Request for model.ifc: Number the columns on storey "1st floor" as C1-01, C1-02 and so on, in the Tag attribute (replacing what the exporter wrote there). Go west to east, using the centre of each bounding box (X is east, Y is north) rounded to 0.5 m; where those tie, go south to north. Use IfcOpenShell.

First a look at what the model holds.

```python
import ifcopenshell
import ifcopenshell.util.element
import ifcopenshell.util.placement

model = ifcopenshell.open("model.ifc")
print(model.schema)
storey = next(s for s in model.by_type("IfcBuildingStorey") if s.Name == "1st floor")
columns = [e for e in ifcopenshell.util.element.get_decomposition(storey) if e.is_a("IfcColumn")]
for e in sorted(columns, key=lambda e: e.id()):
    origin = ifcopenshell.util.placement.get_local_placement(e.ObjectPlacement)[:3, 3]
    print(e.id(), e.Tag, e.Name, origin.round(2) + 0.0, sep=" | ")
```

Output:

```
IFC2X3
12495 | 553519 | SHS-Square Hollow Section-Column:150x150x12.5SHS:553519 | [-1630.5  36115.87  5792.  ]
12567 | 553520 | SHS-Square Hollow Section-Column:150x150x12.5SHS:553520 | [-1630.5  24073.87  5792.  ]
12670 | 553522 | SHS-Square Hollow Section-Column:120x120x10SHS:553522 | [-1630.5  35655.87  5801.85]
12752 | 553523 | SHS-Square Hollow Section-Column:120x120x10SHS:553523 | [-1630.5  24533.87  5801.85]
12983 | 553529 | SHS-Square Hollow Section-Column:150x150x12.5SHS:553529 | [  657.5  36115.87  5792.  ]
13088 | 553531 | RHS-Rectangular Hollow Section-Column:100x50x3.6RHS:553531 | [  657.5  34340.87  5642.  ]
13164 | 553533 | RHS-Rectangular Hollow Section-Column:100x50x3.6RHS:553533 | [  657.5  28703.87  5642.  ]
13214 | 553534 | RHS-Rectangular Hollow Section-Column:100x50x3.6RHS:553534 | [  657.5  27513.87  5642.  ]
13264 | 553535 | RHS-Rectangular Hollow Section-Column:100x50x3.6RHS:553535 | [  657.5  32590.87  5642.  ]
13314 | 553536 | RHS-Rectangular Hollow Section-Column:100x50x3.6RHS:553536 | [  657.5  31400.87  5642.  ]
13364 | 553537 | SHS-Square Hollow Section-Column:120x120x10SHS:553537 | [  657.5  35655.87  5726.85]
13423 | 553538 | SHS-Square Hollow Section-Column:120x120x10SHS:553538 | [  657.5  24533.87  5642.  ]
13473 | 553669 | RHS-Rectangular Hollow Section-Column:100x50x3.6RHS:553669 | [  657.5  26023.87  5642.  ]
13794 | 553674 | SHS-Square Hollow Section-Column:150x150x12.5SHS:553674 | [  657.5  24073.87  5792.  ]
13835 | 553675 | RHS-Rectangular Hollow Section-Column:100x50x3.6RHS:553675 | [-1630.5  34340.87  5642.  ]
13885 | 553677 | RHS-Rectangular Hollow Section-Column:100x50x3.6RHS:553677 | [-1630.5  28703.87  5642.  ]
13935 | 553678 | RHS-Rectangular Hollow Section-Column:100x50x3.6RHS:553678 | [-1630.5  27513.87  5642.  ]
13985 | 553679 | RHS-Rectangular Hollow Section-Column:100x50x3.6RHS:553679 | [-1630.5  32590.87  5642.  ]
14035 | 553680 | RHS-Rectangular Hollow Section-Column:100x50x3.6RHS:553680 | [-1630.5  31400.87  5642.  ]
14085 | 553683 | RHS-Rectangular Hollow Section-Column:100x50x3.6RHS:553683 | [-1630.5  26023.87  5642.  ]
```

```python
import ifcopenshell
import ifcopenshell.geom
import ifcopenshell.util.element
import ifcopenshell.util.shape

model = ifcopenshell.open("model.ifc")
settings = ifcopenshell.geom.settings()
settings.set("use-world-coords", True)


def centre(element):
    shape = ifcopenshell.geom.create_shape(settings, element)
    return ifcopenshell.util.shape.get_bbox_centroid(shape.geometry)


storey = next(s for s in model.by_type("IfcBuildingStorey") if s.Name == "1st floor")
columns = [e for e in ifcopenshell.util.element.get_decomposition(storey) if e.is_a("IfcColumn")]

# Insertion points can sit at a corner or the storey origin, so sort by the geometry (in metres).
centres = {e: centre(e) for e in columns}
columns.sort(key=lambda e: (round(centres[e][0] / 0.5), centres[e][1]))

for i, e in enumerate(columns, start=1):
    number = f"C1-{i:02d}"
    e.Tag = number
    print(e.id(), number)

model.write("model_v2.ifc")
```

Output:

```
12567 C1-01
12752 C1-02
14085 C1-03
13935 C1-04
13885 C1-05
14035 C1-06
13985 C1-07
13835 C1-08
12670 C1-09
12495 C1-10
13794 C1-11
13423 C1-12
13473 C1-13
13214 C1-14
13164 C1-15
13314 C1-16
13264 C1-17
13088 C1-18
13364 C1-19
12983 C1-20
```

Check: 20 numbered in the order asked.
